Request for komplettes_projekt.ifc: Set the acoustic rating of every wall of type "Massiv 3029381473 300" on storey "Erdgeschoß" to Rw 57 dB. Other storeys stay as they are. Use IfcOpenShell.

First a look at what the model holds.

```python
import ifcopenshell
import ifcopenshell.util.element

model = ifcopenshell.open("komplettes_projekt.ifc")
print(model.schema)
storey = next(s for s in model.by_type("IfcBuildingStorey") if s.Name == "Erdgeschoß")
walls = [e for e in ifcopenshell.util.element.get_decomposition(storey) if e.is_a("IfcWall")]
seen = {}
for e in walls:
    element_type = ifcopenshell.util.element.get_type(e)
    key = (element_type.Name if element_type != e and element_type else None, ifcopenshell.util.element.get_pset(e, "Pset_WallCommon", "AcousticRating"))
    seen[key] = seen.get(key, 0) + 1
for (name, value), count in sorted(seen.items(), key=str):
    print(count, "x", name, "|", value)
```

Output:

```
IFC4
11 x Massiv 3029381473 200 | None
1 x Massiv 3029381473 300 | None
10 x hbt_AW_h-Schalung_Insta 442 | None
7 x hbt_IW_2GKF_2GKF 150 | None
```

```python
import ifcopenshell
import ifcopenshell.api.pset
import ifcopenshell.util.element

model = ifcopenshell.open("komplettes_projekt.ifc")

storey = next(s for s in model.by_type("IfcBuildingStorey") if s.Name == "Erdgeschoß")
walls = [e for e in ifcopenshell.util.element.get_decomposition(storey) if e.is_a("IfcWall")]

count = 0
for e in walls:
    element_type = ifcopenshell.util.element.get_type(e)
    if element_type in (None, e) or element_type.Name != "Massiv 3029381473 300":
        continue
    # add_pset returns the element's existing set when there is one.
    pset = ifcopenshell.api.pset.add_pset(model, product=e, name="Pset_WallCommon")
    ifcopenshell.api.pset.edit_pset(model, pset=pset, properties={"AcousticRating": "Rw 57 dB"})
    count += 1

print(count, "walls updated")

model.write("komplettes_projekt_edited.ifc")
```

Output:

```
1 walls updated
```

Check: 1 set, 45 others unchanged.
